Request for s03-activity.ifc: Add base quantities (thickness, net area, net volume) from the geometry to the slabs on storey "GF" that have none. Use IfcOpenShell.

First a look at what the model holds.

```python
import ifcopenshell
import ifcopenshell.util.element
import ifcopenshell.util.unit

model = ifcopenshell.open("s03-activity.ifc")
print(model.schema)
for unit_type in ("LENGTHUNIT", "AREAUNIT", "VOLUMEUNIT"):
    print(unit_type, ifcopenshell.util.unit.calculate_unit_scale(model, unit_type))
storey = next(s for s in model.by_type("IfcBuildingStorey") if s.Name == "GF")
slabs = [e for e in ifcopenshell.util.element.get_decomposition(storey) if e.is_a("IfcSlab")]
for e in sorted(slabs, key=lambda e: e.id()):
    print(e.id(), e.is_a(), e.Name, list(ifcopenshell.util.element.get_psets(e, qtos_only=True)), sep=" | ")
```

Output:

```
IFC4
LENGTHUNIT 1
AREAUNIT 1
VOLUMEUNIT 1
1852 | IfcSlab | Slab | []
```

```python
import ifcopenshell
import ifcopenshell.api.pset
import ifcopenshell.geom
import ifcopenshell.util.element
import ifcopenshell.util.shape
import ifcopenshell.util.unit

model = ifcopenshell.open("s03-activity.ifc")
unit_scale = ifcopenshell.util.unit.calculate_unit_scale(model)
area_scale = ifcopenshell.util.unit.calculate_unit_scale(model, "AREAUNIT")
volume_scale = ifcopenshell.util.unit.calculate_unit_scale(model, "VOLUMEUNIT")
settings = ifcopenshell.geom.settings()

storey = next(s for s in model.by_type("IfcBuildingStorey") if s.Name == "GF")
slabs = [e for e in ifcopenshell.util.element.get_decomposition(storey) if e.is_a("IfcSlab")]

for e in sorted(slabs, key=lambda e: e.id()):
    if ifcopenshell.util.element.get_psets(e, qtos_only=True, should_inherit=False):
        continue
    # Geometry comes back in metres, in the element's own axes.
    shape = ifcopenshell.geom.create_shape(settings, e)
    values = {
        "Width": ifcopenshell.util.shape.get_z(shape.geometry) / unit_scale,
        "NetArea": ifcopenshell.util.shape.get_footprint_area(shape.geometry) / area_scale,
        "NetVolume": ifcopenshell.util.shape.get_volume(shape.geometry) / volume_scale,
    }
    qto = ifcopenshell.api.pset.add_qto(model, product=e, name="Qto_SlabBaseQuantities")
    ifcopenshell.api.pset.edit_qto(model, qto=qto, properties=values)
    print(e.id(), {k: round(v, 3) for k, v in values.items()})

model.write("s03-activity-out.ifc")
```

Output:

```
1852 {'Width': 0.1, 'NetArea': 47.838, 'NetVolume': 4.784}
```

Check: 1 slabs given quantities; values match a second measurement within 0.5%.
